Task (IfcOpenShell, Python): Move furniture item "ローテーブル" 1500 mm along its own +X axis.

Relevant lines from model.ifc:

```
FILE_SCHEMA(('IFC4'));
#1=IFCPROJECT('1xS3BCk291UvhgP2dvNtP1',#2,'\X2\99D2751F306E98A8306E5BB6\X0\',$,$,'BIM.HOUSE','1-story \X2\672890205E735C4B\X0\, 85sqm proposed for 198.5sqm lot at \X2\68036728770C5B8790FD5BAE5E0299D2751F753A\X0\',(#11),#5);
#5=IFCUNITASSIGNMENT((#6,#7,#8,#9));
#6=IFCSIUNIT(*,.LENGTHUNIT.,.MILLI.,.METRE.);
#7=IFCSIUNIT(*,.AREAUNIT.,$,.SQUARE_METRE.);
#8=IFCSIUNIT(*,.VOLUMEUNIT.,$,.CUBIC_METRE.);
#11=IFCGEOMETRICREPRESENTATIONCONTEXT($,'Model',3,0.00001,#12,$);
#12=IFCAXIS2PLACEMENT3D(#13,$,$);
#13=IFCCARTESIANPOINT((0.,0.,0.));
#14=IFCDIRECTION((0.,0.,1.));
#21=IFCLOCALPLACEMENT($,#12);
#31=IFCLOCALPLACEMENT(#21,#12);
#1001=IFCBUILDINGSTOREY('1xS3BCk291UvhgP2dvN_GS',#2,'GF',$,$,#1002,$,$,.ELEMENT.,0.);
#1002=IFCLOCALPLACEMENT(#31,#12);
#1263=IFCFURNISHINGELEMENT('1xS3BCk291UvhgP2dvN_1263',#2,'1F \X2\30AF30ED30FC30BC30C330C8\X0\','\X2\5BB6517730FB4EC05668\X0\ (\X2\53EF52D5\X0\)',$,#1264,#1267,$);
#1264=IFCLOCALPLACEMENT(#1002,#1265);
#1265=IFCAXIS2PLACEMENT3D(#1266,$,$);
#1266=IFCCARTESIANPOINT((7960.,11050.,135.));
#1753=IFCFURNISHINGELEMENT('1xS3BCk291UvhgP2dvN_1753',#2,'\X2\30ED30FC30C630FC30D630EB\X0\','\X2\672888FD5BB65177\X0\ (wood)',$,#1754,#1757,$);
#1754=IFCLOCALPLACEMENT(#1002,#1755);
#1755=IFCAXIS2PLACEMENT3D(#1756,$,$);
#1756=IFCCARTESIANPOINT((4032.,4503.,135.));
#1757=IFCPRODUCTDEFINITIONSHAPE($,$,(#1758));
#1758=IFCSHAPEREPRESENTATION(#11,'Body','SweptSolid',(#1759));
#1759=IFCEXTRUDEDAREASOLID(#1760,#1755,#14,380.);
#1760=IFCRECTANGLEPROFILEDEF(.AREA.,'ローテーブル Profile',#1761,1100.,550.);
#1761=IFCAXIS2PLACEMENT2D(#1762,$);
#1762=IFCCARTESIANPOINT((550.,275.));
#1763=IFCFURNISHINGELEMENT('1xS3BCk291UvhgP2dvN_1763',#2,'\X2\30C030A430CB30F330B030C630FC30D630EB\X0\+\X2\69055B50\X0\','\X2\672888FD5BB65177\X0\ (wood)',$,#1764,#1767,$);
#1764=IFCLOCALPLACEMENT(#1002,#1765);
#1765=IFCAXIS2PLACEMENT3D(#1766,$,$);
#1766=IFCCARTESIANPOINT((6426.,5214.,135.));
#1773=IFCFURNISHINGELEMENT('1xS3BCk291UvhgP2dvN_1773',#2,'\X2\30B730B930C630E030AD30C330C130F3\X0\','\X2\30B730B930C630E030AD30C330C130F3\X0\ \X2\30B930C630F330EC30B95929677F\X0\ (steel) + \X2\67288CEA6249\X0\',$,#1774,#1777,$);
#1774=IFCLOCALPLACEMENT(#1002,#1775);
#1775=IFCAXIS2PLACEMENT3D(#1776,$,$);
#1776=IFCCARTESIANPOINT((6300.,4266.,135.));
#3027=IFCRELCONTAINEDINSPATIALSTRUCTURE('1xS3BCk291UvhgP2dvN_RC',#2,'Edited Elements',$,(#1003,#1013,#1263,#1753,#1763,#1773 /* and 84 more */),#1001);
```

```python
import ifcopenshell
import ifcopenshell.api.geometry
import ifcopenshell.util.placement

model = ifcopenshell.open("model.ifc")

item = model.by_guid("1xS3BCk291UvhgP2dvN_1753")
matrix = ifcopenshell.util.placement.get_local_placement(item.ObjectPlacement)
matrix[:3, 3] += matrix[:3, 0] * 1500.0
ifcopenshell.api.geometry.edit_object_placement(model, product=item, matrix=matrix, is_si=False)

print(ifcopenshell.util.placement.get_local_placement(item.ObjectPlacement).round(3) + 0.0)

model.write("model_updated.ifc")
```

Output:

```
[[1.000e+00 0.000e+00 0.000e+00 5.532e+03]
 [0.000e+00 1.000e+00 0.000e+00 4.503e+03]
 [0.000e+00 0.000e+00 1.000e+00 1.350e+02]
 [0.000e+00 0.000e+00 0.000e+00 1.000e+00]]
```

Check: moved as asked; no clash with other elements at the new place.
